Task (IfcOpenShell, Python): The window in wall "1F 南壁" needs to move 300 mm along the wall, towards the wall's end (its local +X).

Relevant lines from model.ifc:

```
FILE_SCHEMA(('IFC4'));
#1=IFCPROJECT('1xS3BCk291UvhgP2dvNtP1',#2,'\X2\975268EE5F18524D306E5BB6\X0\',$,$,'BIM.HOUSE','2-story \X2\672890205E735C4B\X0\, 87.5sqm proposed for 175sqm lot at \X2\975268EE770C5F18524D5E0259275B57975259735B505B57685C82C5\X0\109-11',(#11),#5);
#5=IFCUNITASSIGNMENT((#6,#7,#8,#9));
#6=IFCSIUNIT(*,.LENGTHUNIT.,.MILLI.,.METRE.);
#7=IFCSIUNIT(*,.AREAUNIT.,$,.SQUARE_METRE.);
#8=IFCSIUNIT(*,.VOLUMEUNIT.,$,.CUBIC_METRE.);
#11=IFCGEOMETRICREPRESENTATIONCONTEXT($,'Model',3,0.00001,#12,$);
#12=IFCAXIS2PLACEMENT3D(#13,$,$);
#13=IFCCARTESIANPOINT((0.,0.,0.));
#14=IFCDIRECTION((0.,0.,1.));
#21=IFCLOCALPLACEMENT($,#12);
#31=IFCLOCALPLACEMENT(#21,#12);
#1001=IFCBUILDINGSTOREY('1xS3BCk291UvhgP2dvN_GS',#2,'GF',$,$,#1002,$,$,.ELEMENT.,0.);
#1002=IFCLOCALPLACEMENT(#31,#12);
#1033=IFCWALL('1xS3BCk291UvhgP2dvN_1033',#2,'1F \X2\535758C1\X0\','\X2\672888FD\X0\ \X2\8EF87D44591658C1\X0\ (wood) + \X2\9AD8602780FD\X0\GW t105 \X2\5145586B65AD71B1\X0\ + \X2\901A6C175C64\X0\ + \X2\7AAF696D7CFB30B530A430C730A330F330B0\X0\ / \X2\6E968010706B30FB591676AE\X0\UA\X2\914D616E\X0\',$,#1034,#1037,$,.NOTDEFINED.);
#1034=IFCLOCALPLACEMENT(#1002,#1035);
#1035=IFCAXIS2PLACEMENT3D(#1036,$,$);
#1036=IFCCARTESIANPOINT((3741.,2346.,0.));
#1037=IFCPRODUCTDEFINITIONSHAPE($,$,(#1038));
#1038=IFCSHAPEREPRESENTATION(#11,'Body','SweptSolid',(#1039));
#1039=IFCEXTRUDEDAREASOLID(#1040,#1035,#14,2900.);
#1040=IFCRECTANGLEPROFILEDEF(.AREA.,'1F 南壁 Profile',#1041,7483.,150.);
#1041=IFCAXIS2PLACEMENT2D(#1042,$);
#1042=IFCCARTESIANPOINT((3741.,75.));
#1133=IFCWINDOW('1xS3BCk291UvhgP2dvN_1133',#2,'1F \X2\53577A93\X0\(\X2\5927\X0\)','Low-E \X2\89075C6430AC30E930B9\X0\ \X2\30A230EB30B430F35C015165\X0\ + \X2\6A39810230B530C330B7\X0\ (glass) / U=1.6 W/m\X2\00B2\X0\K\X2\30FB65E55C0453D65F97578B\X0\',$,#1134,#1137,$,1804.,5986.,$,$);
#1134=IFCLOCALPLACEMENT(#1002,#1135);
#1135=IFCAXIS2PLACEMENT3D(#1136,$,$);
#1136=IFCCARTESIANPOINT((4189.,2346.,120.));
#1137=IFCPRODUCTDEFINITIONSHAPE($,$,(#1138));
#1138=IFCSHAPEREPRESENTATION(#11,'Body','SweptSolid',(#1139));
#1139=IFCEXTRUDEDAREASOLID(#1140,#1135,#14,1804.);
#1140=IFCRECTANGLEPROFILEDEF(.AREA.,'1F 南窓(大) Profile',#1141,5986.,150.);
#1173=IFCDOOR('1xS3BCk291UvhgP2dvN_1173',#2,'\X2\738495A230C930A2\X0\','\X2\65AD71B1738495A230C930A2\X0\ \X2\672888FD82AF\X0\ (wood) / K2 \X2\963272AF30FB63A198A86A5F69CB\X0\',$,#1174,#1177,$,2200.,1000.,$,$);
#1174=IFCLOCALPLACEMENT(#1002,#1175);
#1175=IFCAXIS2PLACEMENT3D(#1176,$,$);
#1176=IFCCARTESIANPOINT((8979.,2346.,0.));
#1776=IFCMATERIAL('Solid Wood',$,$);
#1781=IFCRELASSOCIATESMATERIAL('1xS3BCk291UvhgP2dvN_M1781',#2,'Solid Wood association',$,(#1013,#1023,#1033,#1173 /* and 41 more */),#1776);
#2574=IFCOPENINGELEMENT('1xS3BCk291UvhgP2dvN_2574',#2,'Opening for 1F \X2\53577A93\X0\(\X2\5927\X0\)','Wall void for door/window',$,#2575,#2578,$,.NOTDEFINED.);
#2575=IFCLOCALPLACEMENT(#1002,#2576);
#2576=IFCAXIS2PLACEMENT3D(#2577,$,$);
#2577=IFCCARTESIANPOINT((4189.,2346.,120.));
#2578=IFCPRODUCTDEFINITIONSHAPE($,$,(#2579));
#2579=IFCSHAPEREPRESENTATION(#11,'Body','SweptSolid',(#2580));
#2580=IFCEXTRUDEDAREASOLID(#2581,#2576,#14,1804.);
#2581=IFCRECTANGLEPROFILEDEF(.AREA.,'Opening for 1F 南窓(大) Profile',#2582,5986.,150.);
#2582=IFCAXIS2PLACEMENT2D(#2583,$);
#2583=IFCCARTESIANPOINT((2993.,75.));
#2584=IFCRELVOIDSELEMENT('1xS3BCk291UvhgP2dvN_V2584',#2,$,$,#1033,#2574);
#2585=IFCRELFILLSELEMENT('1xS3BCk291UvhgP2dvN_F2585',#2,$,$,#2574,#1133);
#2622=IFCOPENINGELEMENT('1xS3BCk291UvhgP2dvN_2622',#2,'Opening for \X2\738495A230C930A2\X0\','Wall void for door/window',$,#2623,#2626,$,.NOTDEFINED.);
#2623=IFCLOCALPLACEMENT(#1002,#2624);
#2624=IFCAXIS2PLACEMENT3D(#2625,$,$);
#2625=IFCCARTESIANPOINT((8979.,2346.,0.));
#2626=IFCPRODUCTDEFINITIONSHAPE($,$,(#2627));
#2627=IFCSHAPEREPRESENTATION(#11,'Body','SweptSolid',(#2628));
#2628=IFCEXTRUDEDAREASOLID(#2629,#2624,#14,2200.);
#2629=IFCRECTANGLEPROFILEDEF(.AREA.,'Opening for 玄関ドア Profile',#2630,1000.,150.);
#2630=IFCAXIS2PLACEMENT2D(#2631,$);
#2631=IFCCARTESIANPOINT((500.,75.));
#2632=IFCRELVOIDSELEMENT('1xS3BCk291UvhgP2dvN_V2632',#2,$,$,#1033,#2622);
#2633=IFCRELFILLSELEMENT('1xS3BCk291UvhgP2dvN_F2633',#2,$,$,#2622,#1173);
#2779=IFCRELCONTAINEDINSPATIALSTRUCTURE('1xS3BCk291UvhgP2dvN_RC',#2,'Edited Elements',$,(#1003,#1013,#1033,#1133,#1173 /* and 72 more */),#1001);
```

```python
import ifcopenshell
import ifcopenshell.api.geometry
import ifcopenshell.util.placement
import ifcopenshell.util.unit

model = ifcopenshell.open("model.ifc")
unit_scale = ifcopenshell.util.unit.calculate_unit_scale(model)

window = model.by_guid("1xS3BCk291UvhgP2dvN_1133")
opening = window.FillsVoids[0].RelatingOpeningElement
wall = opening.VoidsElements[0].RelatingBuildingElement

wall_matrix = ifcopenshell.util.placement.get_local_placement(wall.ObjectPlacement)
shift = wall_matrix[:3, 0] * 0.3 / unit_scale
before = ifcopenshell.util.placement.get_local_placement(window.ObjectPlacement)[:3, 3].copy()

# The window is not placed relative to its opening, so move both.
for product in (opening, window):
    matrix = ifcopenshell.util.placement.get_local_placement(product.ObjectPlacement)
    matrix[:3, 3] += shift
    ifcopenshell.api.geometry.edit_object_placement(model, product=product, matrix=matrix, is_si=False)

after = ifcopenshell.util.placement.get_local_placement(window.ObjectPlacement)[:3, 3]
print("window moved by", (after - before).round(3) + 0.0)

model.write("model_v2.ifc")
```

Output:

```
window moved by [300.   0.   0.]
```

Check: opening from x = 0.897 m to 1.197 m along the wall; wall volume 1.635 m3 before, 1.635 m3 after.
